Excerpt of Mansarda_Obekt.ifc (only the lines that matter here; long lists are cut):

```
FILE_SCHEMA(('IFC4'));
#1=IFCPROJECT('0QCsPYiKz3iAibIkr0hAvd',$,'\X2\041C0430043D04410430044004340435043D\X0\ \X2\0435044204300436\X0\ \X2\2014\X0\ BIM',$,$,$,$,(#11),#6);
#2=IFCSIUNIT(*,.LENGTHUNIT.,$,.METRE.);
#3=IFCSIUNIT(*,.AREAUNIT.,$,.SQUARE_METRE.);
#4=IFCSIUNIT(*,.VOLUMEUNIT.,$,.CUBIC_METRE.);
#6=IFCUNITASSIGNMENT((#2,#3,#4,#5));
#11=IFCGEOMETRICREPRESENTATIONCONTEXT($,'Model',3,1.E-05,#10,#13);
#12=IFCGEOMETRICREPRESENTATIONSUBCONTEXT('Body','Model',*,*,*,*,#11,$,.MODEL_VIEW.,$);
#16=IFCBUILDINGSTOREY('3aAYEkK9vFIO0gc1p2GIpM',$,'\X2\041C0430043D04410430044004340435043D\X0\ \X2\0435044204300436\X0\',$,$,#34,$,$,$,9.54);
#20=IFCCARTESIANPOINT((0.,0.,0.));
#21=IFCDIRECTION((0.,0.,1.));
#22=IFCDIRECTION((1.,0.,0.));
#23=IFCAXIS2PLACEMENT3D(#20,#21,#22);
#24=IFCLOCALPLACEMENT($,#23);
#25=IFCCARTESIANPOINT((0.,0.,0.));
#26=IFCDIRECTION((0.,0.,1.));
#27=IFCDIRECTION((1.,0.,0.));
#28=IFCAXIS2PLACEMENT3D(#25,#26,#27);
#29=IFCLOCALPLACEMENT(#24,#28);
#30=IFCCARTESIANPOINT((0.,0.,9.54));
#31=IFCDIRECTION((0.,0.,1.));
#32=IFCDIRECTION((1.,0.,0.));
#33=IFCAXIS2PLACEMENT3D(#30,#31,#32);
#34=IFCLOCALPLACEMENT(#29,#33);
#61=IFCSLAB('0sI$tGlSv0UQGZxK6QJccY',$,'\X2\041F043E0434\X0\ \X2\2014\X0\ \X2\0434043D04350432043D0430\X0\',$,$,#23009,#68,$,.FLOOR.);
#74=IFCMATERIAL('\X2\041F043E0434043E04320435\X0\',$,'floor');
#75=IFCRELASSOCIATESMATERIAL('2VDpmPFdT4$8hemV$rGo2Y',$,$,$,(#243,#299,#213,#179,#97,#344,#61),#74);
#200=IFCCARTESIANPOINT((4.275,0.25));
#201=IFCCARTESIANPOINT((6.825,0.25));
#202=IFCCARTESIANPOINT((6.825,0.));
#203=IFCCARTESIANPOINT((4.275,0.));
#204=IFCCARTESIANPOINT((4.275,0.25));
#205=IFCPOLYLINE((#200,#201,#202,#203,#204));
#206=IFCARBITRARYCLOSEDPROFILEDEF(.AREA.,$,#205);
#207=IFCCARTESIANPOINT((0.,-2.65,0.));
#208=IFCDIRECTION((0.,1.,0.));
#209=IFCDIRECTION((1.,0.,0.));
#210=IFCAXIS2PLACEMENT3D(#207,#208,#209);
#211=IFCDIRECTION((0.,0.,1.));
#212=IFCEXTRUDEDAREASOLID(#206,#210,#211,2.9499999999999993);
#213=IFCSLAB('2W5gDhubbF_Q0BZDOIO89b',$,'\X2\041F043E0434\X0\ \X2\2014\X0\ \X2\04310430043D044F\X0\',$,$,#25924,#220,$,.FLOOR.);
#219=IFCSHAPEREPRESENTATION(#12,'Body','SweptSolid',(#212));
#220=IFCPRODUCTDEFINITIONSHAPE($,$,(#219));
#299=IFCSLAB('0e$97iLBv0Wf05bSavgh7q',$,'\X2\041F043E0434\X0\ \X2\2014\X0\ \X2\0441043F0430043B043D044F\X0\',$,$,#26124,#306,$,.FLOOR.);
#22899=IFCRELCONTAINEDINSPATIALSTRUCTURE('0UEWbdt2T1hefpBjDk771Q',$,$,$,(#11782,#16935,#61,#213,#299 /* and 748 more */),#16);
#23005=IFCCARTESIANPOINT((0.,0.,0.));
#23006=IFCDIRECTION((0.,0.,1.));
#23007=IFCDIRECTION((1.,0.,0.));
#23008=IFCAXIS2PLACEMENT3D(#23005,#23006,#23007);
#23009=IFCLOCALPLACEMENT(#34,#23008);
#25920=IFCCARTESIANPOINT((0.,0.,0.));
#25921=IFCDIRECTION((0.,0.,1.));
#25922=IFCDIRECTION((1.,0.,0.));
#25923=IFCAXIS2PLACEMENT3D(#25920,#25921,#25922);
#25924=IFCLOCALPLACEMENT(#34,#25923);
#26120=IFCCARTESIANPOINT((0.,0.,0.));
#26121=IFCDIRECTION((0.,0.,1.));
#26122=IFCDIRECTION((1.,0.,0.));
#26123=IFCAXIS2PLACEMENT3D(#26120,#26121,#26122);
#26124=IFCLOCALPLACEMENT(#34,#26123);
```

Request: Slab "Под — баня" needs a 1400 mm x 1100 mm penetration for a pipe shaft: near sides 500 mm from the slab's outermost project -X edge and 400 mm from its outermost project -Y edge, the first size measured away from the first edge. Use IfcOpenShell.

```python
import numpy as np
import ifcopenshell
import ifcopenshell.api.feature
import ifcopenshell.api.geometry
import ifcopenshell.api.root
import ifcopenshell.geom
import ifcopenshell.util.placement
import ifcopenshell.util.representation
import ifcopenshell.util.shape
import ifcopenshell.util.unit

model = ifcopenshell.open("Mansarda_Obekt.ifc")
unit_scale = ifcopenshell.util.unit.calculate_unit_scale(model)
settings = ifcopenshell.geom.settings()


def volume(element):
    """Net volume in cubic metres, openings subtracted."""
    shape = ifcopenshell.geom.create_shape(settings, element)
    return ifcopenshell.util.shape.get_volume(shape.geometry)


slab = model.by_guid("2W5gDhubbF_Q0BZDOIO89b")
before = volume(slab)

# Extent in the slab's own axes, in metres. The edges named are its -X and -Y sides.
slab_shape = ifcopenshell.geom.create_shape(settings, slab)
vertices = ifcopenshell.util.shape.get_vertices(slab_shape.geometry)
x_min, y_min, bottom = vertices.min(axis=0)
top = vertices[:, 2].max()

opening = ifcopenshell.api.root.create_entity(model, ifc_class="IfcOpeningElement", name="Pipe shaft opening", predefined_type="OPENING")
context = ifcopenshell.util.representation.get_context(model, "Model", "Body", "MODEL_VIEW")
width, depth = 1.4, 1.1
outline = [(0.0, 0.0), (width, 0.0), (width, depth), (0.0, depth), (0.0, 0.0)]
# Overshoot both faces by 50 mm so the cut is clean.
shape = ifcopenshell.api.geometry.add_slab_representation(
    model, context=context, depth=top - bottom + 0.1, polyline=outline
)
ifcopenshell.api.geometry.assign_representation(model, product=opening, representation=shape)

matrix = ifcopenshell.util.placement.get_local_placement(slab.ObjectPlacement)
matrix[:, 3] = matrix @ np.append(np.array([x_min + 0.5, y_min + 0.4, bottom - 0.05]) / unit_scale, 1.0)
ifcopenshell.api.geometry.edit_object_placement(model, product=opening, matrix=matrix, is_si=False)
ifcopenshell.api.feature.add_feature(model, feature=opening, element=slab)

after = volume(slab)

print(f"slab volume {before:.3f} -> {after:.3f} m3")

model.write("Mansarda_Obekt_updated.ifc")
```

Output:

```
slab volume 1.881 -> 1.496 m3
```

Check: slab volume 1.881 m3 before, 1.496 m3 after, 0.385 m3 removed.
